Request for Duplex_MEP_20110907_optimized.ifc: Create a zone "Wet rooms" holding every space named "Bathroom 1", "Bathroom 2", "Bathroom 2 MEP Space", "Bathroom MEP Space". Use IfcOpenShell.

First a look at what the model holds.

```python
import ifcopenshell

model = ifcopenshell.open("Duplex_MEP_20110907_optimized.ifc")
print(model.schema)
seen = {}
for space in model.by_type("IfcSpace"):
    seen[space.LongName] = seen.get(space.LongName, 0) + 1
for name, count in sorted(seen.items(), key=str):
    print(count, "x", name)
print("zones:", [z.Name for z in model.by_type("IfcZone")][:20])
```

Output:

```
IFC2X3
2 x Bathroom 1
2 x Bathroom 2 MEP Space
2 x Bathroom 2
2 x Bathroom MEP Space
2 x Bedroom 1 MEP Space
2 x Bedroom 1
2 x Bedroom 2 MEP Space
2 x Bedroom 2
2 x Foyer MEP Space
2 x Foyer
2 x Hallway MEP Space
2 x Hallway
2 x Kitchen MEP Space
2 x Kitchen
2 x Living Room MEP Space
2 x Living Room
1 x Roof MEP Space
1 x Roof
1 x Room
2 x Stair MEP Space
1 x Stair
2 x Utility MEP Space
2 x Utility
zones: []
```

```python
import ifcopenshell
import ifcopenshell.api.group
import ifcopenshell.api.root

model = ifcopenshell.open("Duplex_MEP_20110907_optimized.ifc")

names = {"Bathroom 1", "Bathroom 2", "Bathroom 2 MEP Space", "Bathroom MEP Space"}
spaces = [s for s in model.by_type("IfcSpace") if s.LongName in names]

zone = ifcopenshell.api.root.create_entity(model, ifc_class="IfcZone", name="Wet rooms")
ifcopenshell.api.group.assign_group(model, products=spaces, group=zone)
print(len(spaces), "spaces in", zone.Name)

model.write("Duplex_MEP_20110907_optimized_rev.ifc")
```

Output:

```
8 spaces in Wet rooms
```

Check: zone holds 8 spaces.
